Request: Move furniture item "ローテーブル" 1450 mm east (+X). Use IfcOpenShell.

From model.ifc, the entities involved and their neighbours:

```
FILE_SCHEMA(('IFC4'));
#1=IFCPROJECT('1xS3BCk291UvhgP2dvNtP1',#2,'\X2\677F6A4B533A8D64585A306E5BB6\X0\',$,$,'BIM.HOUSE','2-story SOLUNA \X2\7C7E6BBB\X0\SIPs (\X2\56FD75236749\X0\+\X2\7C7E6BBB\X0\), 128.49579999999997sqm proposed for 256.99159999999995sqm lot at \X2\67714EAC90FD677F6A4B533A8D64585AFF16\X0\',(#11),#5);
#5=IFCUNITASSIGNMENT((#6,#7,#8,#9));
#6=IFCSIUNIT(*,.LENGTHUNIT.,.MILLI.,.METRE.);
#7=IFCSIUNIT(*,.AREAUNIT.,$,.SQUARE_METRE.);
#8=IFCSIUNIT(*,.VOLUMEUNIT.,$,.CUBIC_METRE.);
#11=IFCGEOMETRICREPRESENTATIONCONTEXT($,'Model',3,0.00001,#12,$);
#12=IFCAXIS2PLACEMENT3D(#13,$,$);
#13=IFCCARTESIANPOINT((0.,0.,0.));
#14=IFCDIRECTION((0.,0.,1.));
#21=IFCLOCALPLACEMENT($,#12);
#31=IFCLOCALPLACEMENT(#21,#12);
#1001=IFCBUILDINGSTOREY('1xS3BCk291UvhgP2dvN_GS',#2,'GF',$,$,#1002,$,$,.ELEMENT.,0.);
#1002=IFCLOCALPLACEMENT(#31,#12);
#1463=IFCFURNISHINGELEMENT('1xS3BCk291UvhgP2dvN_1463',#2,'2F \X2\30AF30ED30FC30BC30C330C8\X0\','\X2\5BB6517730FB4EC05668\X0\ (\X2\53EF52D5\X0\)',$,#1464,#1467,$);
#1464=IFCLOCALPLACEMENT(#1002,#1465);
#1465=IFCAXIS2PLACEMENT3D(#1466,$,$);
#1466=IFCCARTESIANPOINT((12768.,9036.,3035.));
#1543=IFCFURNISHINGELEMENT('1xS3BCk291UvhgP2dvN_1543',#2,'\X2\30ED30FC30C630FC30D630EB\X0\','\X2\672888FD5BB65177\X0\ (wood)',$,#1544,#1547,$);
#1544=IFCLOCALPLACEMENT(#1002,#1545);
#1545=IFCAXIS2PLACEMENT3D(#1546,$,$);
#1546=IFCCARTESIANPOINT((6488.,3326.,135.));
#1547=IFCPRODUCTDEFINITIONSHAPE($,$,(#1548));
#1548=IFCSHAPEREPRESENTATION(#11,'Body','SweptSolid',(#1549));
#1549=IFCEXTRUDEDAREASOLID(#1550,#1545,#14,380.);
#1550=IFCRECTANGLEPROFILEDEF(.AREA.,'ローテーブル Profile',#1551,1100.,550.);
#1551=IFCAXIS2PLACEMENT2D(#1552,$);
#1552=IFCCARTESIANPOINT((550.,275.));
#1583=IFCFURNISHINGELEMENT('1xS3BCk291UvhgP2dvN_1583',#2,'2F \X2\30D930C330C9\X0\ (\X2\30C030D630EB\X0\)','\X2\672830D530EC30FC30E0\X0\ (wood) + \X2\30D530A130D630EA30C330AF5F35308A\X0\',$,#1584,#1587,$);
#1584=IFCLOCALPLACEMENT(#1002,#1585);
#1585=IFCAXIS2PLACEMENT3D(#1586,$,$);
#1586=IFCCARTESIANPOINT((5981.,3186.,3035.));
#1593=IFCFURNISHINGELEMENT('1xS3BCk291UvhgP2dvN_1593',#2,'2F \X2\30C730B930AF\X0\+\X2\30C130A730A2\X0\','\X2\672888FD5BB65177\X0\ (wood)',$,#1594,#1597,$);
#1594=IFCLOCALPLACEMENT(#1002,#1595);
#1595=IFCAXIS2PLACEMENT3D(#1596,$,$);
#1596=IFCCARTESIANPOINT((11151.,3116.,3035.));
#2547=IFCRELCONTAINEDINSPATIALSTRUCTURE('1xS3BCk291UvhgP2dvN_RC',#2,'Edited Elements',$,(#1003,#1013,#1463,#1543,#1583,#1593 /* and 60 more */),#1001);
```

```python
import ifcopenshell
import ifcopenshell.api.geometry
import ifcopenshell.util.placement

model = ifcopenshell.open("model.ifc")

item = model.by_id(1543)
matrix = ifcopenshell.util.placement.get_local_placement(item.ObjectPlacement)
matrix[0, 3] += 1450.0
ifcopenshell.api.geometry.edit_object_placement(model, product=item, matrix=matrix, is_si=False)

print(ifcopenshell.util.placement.get_local_placement(item.ObjectPlacement).round(3) + 0.0)

model.write("model_updated.ifc")
```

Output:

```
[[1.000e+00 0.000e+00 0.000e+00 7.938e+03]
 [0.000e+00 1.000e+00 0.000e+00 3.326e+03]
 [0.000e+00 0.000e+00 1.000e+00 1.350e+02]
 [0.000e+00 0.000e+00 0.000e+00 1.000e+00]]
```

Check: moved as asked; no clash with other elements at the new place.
